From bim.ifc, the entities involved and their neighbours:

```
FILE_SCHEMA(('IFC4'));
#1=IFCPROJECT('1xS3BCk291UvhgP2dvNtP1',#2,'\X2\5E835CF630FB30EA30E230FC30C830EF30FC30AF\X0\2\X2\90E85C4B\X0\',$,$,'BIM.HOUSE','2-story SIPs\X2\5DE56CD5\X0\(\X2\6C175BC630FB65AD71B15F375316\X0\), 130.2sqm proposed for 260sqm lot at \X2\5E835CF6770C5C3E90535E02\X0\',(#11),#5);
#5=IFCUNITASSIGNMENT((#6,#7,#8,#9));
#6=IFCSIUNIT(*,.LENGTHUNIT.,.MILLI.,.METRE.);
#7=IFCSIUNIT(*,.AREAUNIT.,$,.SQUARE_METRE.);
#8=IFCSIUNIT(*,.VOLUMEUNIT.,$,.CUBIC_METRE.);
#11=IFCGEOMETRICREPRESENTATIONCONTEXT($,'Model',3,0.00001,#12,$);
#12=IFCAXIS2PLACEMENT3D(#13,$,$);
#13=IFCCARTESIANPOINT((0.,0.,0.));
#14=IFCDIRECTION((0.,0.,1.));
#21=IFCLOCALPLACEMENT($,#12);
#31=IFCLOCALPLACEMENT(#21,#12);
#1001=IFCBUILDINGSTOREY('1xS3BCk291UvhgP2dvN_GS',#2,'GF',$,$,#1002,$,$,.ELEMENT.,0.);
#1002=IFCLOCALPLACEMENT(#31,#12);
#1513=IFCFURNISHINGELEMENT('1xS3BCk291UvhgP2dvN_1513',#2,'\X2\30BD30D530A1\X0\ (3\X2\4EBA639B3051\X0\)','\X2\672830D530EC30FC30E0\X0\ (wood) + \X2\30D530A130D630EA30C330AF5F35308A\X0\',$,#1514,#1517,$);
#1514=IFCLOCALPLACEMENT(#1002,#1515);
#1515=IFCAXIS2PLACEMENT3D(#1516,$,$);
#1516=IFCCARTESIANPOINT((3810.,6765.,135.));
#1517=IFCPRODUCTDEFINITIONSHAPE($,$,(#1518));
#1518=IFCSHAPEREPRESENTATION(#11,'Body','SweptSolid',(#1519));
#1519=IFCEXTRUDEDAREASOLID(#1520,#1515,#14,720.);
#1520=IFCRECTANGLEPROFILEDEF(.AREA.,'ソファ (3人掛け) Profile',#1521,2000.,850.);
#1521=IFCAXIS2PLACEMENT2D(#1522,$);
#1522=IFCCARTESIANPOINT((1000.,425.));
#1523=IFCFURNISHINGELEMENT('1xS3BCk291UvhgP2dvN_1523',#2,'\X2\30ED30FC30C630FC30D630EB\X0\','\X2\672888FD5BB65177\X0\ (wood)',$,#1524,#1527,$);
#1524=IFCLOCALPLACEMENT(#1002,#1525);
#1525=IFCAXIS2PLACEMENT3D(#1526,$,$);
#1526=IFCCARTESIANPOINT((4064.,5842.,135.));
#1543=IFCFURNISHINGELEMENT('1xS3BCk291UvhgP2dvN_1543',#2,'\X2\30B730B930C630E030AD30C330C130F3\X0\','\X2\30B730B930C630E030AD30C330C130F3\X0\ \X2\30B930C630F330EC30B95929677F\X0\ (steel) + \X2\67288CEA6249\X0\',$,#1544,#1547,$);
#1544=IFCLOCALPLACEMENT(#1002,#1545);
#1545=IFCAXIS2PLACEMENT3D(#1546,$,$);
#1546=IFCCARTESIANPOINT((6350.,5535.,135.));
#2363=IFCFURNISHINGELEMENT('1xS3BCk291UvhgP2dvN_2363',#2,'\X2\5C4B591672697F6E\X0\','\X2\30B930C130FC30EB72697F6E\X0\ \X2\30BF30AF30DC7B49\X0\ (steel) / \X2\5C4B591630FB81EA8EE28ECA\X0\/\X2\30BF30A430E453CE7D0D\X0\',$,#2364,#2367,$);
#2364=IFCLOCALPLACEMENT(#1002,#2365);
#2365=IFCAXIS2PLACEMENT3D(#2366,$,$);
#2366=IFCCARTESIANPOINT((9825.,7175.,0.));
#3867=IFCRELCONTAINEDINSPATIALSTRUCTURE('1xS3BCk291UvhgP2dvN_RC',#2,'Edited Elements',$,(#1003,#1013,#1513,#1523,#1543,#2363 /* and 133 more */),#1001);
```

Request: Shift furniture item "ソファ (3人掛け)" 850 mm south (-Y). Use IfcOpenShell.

```python
import ifcopenshell
import ifcopenshell.api.geometry
import ifcopenshell.util.placement
import ifcopenshell.util.unit

model = ifcopenshell.open("bim.ifc")
unit_scale = ifcopenshell.util.unit.calculate_unit_scale(model)

item = model.by_guid("1xS3BCk291UvhgP2dvN_1513")
matrix = ifcopenshell.util.placement.get_local_placement(item.ObjectPlacement)
matrix[1, 3] -= 0.85 / unit_scale
ifcopenshell.api.geometry.edit_object_placement(model, product=item, matrix=matrix, is_si=False)

print(ifcopenshell.util.placement.get_local_placement(item.ObjectPlacement).round(3) + 0.0)

model.write("bim_updated.ifc")
```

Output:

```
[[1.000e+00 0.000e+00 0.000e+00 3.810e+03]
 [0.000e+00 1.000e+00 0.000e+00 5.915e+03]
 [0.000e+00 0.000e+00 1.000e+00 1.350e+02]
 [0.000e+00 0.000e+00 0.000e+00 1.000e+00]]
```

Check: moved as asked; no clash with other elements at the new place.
